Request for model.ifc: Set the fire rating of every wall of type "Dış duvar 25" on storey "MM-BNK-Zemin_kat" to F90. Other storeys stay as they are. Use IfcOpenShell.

First a look at what the model holds.

```python
import ifcopenshell
import ifcopenshell.util.element

model = ifcopenshell.open("model.ifc")
print(model.schema)
storey = next(s for s in model.by_type("IfcBuildingStorey") if s.Name == "MM-BNK-Zemin_kat")
walls = [e for e in ifcopenshell.util.element.get_decomposition(storey) if e.is_a("IfcWall")]
seen = {}
for e in walls:
    element_type = ifcopenshell.util.element.get_type(e)
    key = (element_type.Name if element_type != e and element_type else None, ifcopenshell.util.element.get_pset(e, "Pset_WallCommon", "FireRating"))
    seen[key] = seen.get(key, 0) + 1
for (name, value), count in sorted(seen.items(), key=str):
    print(count, "x", name, "|", value)
```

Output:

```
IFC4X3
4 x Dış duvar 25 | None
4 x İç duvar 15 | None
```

```python
import ifcopenshell
import ifcopenshell.api.pset
import ifcopenshell.util.element

model = ifcopenshell.open("model.ifc")

storey = next(s for s in model.by_type("IfcBuildingStorey") if s.Name == "MM-BNK-Zemin_kat")
walls = [e for e in ifcopenshell.util.element.get_decomposition(storey) if e.is_a("IfcWall")]

count = 0
for e in walls:
    element_type = ifcopenshell.util.element.get_type(e)
    if element_type in (None, e) or element_type.Name != "Dış duvar 25":
        continue
    # add_pset returns the element's existing set when there is one.
    pset = ifcopenshell.api.pset.add_pset(model, product=e, name="Pset_WallCommon")
    ifcopenshell.api.pset.edit_pset(model, pset=pset, properties={"FireRating": "F90"})
    count += 1

print(count, "walls updated")

model.write("model_updated.ifc")
```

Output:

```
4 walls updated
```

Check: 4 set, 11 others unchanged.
